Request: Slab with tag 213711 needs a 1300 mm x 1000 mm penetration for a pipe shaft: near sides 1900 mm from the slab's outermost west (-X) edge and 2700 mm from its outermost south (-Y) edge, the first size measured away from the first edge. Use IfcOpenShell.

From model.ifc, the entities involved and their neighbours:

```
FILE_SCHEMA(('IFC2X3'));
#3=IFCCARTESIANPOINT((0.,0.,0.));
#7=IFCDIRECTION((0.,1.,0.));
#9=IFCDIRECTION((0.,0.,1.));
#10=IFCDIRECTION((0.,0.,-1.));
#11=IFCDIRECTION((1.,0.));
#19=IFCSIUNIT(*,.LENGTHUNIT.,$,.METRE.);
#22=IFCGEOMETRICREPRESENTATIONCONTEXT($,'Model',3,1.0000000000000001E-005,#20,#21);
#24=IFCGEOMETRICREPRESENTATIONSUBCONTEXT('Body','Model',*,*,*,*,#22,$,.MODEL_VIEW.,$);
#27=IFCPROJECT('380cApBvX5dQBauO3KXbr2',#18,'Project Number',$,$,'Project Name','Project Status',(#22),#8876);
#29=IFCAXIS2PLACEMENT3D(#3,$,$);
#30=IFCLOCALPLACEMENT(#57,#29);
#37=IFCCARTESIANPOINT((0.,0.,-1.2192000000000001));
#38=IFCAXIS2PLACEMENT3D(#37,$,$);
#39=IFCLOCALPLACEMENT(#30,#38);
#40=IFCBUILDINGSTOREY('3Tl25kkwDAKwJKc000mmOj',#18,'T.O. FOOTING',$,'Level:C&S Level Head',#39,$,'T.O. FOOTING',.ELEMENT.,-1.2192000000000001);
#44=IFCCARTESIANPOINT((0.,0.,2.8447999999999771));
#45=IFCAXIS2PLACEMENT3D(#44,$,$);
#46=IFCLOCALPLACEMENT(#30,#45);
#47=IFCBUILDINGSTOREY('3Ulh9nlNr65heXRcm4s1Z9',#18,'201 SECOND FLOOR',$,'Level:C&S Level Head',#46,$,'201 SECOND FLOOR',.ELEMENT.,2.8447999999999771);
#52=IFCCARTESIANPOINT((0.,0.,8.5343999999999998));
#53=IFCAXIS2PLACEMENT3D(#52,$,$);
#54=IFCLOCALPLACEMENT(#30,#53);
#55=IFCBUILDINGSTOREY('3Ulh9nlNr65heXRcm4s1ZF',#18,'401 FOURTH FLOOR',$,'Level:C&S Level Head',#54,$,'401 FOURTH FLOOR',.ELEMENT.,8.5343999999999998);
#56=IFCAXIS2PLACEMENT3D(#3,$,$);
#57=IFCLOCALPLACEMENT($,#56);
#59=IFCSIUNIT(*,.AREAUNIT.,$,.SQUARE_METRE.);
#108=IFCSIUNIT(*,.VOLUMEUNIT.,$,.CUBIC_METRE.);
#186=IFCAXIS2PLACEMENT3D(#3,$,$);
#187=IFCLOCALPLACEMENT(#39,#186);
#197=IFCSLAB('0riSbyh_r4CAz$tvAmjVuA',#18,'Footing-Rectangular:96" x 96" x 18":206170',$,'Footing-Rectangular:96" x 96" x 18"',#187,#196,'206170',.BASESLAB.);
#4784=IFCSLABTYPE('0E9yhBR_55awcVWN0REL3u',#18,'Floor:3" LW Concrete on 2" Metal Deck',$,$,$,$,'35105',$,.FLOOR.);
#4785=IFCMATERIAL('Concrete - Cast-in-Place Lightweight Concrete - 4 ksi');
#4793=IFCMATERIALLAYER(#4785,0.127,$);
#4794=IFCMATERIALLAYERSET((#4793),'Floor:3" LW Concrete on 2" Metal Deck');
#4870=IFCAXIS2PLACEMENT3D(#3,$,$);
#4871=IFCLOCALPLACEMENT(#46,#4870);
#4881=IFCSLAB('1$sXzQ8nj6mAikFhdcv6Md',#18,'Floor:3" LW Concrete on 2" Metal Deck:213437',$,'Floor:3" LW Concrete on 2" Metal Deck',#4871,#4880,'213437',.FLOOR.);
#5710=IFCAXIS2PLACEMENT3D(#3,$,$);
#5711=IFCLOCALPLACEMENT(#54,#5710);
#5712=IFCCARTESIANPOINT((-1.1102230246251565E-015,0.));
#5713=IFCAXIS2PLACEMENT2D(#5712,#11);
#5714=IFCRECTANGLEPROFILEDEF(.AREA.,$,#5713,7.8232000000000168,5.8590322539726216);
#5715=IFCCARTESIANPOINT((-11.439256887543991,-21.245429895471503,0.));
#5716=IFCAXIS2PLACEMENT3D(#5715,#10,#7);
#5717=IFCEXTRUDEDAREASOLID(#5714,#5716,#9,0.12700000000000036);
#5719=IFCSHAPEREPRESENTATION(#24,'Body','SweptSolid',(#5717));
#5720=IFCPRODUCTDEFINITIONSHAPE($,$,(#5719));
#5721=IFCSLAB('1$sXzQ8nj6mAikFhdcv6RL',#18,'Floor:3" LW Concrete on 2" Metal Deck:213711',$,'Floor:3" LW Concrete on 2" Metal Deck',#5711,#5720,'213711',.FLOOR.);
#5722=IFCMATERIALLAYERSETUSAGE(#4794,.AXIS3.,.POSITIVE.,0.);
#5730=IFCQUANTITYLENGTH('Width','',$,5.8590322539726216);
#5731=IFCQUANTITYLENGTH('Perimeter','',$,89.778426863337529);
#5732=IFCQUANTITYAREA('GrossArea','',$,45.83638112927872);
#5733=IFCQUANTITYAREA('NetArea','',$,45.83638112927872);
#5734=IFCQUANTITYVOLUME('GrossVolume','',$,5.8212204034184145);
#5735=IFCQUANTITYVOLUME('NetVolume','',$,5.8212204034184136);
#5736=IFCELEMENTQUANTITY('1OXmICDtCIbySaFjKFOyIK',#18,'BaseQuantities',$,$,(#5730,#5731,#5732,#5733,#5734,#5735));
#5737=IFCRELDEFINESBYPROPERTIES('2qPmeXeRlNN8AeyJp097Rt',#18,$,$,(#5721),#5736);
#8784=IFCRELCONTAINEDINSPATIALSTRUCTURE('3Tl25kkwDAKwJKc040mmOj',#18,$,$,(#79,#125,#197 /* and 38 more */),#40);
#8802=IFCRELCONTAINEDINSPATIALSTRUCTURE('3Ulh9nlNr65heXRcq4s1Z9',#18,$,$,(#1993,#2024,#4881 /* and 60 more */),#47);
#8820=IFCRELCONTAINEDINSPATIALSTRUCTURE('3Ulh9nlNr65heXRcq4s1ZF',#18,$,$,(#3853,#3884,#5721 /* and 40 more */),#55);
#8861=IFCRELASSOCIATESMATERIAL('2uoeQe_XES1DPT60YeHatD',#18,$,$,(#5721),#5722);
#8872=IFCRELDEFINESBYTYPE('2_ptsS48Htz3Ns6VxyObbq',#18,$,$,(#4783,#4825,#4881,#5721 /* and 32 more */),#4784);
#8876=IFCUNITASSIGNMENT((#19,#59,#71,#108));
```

```python
import numpy as np
import ifcopenshell
import ifcopenshell.api.feature
import ifcopenshell.api.geometry
import ifcopenshell.api.pset
import ifcopenshell.api.root
import ifcopenshell.geom
import ifcopenshell.util.element
import ifcopenshell.util.placement
import ifcopenshell.util.representation
import ifcopenshell.util.shape
import ifcopenshell.util.unit

model = ifcopenshell.open("model.ifc")
unit_scale = ifcopenshell.util.unit.calculate_unit_scale(model)
area_scale = ifcopenshell.util.unit.calculate_unit_scale(model, "AREAUNIT")
volume_scale = ifcopenshell.util.unit.calculate_unit_scale(model, "VOLUMEUNIT")
settings = ifcopenshell.geom.settings()


def volume(element):
    """Net volume in cubic metres, openings subtracted."""
    shape = ifcopenshell.geom.create_shape(settings, element)
    return ifcopenshell.util.shape.get_volume(shape.geometry)


slab = model.by_guid("1$sXzQ8nj6mAikFhdcv6RL")
before = volume(slab)

# Extent in the slab's own axes, in metres. The edges named are its -X and -Y sides.
slab_shape = ifcopenshell.geom.create_shape(settings, slab)
vertices = ifcopenshell.util.shape.get_vertices(slab_shape.geometry)
x_min, y_min, bottom = vertices.min(axis=0)
top = vertices[:, 2].max()

opening = ifcopenshell.api.root.create_entity(model, ifc_class="IfcOpeningElement", name="Pipe shaft opening")
context = ifcopenshell.util.representation.get_context(model, "Model", "Body", "MODEL_VIEW")
width, depth = 1.3, 1
outline = [(0.0, 0.0), (width, 0.0), (width, depth), (0.0, depth), (0.0, 0.0)]
# Overshoot both faces by 50 mm so the cut is clean.
shape = ifcopenshell.api.geometry.add_slab_representation(
    model, context=context, depth=top - bottom + 0.1, polyline=outline
)
ifcopenshell.api.geometry.assign_representation(model, product=opening, representation=shape)

matrix = ifcopenshell.util.placement.get_local_placement(slab.ObjectPlacement)
matrix[:, 3] = matrix @ np.append(np.array([x_min + 1.9, y_min + 2.7, bottom - 0.05]) / unit_scale, 1.0)
ifcopenshell.api.geometry.edit_object_placement(model, product=opening, matrix=matrix, is_si=False)
ifcopenshell.api.feature.add_feature(model, feature=opening, element=slab)

after = volume(slab)

# Update the slab's stored quantities.
qto = model.by_id(ifcopenshell.util.element.get_pset(slab, "BaseQuantities", should_inherit=False)["id"])
ifcopenshell.api.pset.edit_qto(model, qto=qto, properties={
    "NetArea": after / (top - bottom) / area_scale,
    "NetVolume": after / volume_scale,
})

print(f"slab volume {before:.3f} -> {after:.3f} m3")

model.write("model_v2.ifc")
```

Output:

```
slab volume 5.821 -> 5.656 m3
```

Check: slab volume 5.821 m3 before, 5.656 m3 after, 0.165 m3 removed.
